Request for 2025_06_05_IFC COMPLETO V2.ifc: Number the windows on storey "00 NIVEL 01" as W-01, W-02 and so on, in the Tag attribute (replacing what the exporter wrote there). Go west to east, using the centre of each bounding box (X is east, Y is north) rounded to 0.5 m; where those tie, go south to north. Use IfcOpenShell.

First a look at what the model holds.

```python
import ifcopenshell
import ifcopenshell.util.element
import ifcopenshell.util.placement

model = ifcopenshell.open("2025_06_05_IFC COMPLETO V2.ifc")
print(model.schema)
storey = next(s for s in model.by_type("IfcBuildingStorey") if s.Name == "00 NIVEL 01")
windows = [e for e in ifcopenshell.util.element.get_decomposition(storey) if e.is_a("IfcWindow")]
for e in sorted(windows, key=lambda e: e.id()):
    origin = ifcopenshell.util.placement.get_local_placement(e.ObjectPlacement)[:3, 3]
    print(e.id(), e.Tag, e.Name, origin.round(2) + 0.0, sep=" | ")
```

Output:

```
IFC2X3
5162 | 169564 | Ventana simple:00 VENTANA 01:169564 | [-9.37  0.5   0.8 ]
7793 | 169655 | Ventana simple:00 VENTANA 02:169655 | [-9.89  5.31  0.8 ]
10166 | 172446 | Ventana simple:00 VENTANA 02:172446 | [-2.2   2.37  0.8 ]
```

```python
import ifcopenshell
import ifcopenshell.geom
import ifcopenshell.util.element
import ifcopenshell.util.shape

model = ifcopenshell.open("2025_06_05_IFC COMPLETO V2.ifc")
settings = ifcopenshell.geom.settings()
settings.set("use-world-coords", True)


def centre(element):
    shape = ifcopenshell.geom.create_shape(settings, element)
    return ifcopenshell.util.shape.get_bbox_centroid(shape.geometry)


storey = next(s for s in model.by_type("IfcBuildingStorey") if s.Name == "00 NIVEL 01")
windows = [e for e in ifcopenshell.util.element.get_decomposition(storey) if e.is_a("IfcWindow")]

# Insertion points can sit at a corner or the storey origin, so sort by the geometry (in metres).
centres = {e: centre(e) for e in windows}
windows.sort(key=lambda e: (round(centres[e][0] / 0.5), centres[e][1]))

for i, e in enumerate(windows, start=1):
    number = f"W-{i:02d}"
    e.Tag = number
    print(e.id(), number)

model.write("2025_06_05_IFC COMPLETO V2-out.ifc")
```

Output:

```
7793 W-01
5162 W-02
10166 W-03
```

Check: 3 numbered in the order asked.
